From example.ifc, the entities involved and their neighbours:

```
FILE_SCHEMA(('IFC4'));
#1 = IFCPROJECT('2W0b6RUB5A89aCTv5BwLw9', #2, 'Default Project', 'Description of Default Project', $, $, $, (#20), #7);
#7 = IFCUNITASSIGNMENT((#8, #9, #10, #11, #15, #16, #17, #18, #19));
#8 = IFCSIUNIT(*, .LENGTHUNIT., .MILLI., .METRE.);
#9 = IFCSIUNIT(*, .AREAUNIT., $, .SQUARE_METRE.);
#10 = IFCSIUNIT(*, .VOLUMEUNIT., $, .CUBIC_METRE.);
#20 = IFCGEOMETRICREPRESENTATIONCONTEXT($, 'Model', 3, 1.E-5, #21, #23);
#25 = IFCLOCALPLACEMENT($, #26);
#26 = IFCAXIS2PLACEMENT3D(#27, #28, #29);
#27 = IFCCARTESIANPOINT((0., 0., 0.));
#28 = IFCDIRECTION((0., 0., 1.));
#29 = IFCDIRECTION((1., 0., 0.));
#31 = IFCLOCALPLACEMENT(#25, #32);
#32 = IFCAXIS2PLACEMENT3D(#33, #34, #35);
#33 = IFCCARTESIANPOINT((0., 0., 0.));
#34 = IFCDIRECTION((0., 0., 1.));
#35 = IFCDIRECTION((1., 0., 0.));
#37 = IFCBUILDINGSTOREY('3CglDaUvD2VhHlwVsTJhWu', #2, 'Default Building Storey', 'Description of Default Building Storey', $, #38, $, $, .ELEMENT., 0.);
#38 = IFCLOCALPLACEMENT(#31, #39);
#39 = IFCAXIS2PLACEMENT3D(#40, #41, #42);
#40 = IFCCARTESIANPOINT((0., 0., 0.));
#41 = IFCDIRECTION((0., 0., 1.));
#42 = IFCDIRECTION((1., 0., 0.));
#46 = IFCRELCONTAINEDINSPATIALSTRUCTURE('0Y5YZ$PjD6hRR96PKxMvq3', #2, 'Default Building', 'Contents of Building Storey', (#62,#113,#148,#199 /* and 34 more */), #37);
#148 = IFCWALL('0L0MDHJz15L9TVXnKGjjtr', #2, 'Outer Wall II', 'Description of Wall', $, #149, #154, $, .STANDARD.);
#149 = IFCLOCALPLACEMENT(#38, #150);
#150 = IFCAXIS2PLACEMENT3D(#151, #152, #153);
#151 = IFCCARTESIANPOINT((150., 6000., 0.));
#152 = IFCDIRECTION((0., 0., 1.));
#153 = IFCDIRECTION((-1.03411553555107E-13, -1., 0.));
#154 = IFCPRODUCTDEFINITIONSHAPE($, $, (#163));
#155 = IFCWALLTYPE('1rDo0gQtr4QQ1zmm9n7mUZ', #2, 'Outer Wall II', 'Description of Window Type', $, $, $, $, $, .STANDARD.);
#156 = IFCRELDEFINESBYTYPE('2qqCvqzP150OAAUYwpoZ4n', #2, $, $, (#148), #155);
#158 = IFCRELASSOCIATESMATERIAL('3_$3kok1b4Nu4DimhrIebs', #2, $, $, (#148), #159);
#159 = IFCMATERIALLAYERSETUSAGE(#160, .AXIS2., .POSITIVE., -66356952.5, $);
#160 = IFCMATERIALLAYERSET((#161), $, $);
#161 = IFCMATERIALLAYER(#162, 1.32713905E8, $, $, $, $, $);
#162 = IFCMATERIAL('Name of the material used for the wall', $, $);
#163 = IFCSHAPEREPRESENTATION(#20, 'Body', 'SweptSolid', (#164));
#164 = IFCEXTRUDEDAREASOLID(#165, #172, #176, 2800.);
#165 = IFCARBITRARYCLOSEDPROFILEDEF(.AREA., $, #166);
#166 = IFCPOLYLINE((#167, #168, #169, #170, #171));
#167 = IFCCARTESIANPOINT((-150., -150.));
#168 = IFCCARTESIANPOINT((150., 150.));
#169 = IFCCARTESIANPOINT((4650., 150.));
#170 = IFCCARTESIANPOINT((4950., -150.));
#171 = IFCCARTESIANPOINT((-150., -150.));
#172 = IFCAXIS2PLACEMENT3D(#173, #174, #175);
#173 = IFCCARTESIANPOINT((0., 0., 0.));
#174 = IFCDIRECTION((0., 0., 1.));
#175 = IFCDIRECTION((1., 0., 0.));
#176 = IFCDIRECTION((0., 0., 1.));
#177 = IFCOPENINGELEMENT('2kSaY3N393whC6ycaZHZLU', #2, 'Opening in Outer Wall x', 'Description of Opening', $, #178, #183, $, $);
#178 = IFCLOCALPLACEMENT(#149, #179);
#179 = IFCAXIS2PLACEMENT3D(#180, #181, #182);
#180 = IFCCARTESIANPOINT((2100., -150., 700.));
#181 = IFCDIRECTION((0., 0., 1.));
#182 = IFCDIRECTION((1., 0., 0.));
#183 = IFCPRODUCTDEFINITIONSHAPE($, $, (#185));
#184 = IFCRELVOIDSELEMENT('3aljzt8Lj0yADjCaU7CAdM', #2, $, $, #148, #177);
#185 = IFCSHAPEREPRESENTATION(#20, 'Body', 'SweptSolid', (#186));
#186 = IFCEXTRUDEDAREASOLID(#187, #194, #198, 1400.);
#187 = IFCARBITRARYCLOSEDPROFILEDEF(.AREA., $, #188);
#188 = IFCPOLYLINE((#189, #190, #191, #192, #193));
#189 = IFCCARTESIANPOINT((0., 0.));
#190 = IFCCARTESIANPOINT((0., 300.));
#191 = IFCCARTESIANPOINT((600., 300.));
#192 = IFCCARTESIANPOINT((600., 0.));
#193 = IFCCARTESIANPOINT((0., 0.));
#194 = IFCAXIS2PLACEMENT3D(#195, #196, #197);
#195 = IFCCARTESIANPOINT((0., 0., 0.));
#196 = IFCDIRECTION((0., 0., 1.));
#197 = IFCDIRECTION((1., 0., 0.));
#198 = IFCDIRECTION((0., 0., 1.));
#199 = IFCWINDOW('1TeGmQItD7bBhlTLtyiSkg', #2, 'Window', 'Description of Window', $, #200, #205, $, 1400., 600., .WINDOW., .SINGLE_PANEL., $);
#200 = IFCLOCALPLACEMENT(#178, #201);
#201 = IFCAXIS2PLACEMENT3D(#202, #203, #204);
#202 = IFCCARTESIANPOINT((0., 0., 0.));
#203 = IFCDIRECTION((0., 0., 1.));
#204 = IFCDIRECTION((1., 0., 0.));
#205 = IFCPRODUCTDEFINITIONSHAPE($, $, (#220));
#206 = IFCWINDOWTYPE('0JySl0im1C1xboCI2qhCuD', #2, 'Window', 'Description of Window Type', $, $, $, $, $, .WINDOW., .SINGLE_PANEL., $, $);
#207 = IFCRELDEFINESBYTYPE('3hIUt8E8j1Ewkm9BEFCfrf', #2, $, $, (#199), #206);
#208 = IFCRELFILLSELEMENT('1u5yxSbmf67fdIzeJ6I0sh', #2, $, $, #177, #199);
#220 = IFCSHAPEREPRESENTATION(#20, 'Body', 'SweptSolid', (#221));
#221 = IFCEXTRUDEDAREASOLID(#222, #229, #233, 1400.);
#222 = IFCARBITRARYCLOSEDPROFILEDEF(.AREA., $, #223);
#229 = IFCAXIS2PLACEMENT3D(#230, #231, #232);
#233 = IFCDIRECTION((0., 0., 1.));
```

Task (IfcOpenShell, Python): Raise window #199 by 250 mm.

```python
import numpy as np
import ifcopenshell
import ifcopenshell.api.geometry
import ifcopenshell.util.placement
import ifcopenshell.util.unit

model = ifcopenshell.open("example.ifc")
unit_scale = ifcopenshell.util.unit.calculate_unit_scale(model)

window = model.by_guid("1TeGmQItD7bBhlTLtyiSkg")
opening = window.FillsVoids[0].RelatingOpeningElement
dz = 250.0

shift = np.array([0.0, 0.0, dz])
# The window is placed relative to its opening, so it follows when the opening moves.
matrix = ifcopenshell.util.placement.get_local_placement(opening.ObjectPlacement)
matrix[:3, 3] += shift
ifcopenshell.api.geometry.edit_object_placement(
    model, product=opening, matrix=matrix, is_si=False, should_transform_children=True
)

print(f"moved by {dz * unit_scale:+.3f} m")

model.write("example_edited.ifc")
```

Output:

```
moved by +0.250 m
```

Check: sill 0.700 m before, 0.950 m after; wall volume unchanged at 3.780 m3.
